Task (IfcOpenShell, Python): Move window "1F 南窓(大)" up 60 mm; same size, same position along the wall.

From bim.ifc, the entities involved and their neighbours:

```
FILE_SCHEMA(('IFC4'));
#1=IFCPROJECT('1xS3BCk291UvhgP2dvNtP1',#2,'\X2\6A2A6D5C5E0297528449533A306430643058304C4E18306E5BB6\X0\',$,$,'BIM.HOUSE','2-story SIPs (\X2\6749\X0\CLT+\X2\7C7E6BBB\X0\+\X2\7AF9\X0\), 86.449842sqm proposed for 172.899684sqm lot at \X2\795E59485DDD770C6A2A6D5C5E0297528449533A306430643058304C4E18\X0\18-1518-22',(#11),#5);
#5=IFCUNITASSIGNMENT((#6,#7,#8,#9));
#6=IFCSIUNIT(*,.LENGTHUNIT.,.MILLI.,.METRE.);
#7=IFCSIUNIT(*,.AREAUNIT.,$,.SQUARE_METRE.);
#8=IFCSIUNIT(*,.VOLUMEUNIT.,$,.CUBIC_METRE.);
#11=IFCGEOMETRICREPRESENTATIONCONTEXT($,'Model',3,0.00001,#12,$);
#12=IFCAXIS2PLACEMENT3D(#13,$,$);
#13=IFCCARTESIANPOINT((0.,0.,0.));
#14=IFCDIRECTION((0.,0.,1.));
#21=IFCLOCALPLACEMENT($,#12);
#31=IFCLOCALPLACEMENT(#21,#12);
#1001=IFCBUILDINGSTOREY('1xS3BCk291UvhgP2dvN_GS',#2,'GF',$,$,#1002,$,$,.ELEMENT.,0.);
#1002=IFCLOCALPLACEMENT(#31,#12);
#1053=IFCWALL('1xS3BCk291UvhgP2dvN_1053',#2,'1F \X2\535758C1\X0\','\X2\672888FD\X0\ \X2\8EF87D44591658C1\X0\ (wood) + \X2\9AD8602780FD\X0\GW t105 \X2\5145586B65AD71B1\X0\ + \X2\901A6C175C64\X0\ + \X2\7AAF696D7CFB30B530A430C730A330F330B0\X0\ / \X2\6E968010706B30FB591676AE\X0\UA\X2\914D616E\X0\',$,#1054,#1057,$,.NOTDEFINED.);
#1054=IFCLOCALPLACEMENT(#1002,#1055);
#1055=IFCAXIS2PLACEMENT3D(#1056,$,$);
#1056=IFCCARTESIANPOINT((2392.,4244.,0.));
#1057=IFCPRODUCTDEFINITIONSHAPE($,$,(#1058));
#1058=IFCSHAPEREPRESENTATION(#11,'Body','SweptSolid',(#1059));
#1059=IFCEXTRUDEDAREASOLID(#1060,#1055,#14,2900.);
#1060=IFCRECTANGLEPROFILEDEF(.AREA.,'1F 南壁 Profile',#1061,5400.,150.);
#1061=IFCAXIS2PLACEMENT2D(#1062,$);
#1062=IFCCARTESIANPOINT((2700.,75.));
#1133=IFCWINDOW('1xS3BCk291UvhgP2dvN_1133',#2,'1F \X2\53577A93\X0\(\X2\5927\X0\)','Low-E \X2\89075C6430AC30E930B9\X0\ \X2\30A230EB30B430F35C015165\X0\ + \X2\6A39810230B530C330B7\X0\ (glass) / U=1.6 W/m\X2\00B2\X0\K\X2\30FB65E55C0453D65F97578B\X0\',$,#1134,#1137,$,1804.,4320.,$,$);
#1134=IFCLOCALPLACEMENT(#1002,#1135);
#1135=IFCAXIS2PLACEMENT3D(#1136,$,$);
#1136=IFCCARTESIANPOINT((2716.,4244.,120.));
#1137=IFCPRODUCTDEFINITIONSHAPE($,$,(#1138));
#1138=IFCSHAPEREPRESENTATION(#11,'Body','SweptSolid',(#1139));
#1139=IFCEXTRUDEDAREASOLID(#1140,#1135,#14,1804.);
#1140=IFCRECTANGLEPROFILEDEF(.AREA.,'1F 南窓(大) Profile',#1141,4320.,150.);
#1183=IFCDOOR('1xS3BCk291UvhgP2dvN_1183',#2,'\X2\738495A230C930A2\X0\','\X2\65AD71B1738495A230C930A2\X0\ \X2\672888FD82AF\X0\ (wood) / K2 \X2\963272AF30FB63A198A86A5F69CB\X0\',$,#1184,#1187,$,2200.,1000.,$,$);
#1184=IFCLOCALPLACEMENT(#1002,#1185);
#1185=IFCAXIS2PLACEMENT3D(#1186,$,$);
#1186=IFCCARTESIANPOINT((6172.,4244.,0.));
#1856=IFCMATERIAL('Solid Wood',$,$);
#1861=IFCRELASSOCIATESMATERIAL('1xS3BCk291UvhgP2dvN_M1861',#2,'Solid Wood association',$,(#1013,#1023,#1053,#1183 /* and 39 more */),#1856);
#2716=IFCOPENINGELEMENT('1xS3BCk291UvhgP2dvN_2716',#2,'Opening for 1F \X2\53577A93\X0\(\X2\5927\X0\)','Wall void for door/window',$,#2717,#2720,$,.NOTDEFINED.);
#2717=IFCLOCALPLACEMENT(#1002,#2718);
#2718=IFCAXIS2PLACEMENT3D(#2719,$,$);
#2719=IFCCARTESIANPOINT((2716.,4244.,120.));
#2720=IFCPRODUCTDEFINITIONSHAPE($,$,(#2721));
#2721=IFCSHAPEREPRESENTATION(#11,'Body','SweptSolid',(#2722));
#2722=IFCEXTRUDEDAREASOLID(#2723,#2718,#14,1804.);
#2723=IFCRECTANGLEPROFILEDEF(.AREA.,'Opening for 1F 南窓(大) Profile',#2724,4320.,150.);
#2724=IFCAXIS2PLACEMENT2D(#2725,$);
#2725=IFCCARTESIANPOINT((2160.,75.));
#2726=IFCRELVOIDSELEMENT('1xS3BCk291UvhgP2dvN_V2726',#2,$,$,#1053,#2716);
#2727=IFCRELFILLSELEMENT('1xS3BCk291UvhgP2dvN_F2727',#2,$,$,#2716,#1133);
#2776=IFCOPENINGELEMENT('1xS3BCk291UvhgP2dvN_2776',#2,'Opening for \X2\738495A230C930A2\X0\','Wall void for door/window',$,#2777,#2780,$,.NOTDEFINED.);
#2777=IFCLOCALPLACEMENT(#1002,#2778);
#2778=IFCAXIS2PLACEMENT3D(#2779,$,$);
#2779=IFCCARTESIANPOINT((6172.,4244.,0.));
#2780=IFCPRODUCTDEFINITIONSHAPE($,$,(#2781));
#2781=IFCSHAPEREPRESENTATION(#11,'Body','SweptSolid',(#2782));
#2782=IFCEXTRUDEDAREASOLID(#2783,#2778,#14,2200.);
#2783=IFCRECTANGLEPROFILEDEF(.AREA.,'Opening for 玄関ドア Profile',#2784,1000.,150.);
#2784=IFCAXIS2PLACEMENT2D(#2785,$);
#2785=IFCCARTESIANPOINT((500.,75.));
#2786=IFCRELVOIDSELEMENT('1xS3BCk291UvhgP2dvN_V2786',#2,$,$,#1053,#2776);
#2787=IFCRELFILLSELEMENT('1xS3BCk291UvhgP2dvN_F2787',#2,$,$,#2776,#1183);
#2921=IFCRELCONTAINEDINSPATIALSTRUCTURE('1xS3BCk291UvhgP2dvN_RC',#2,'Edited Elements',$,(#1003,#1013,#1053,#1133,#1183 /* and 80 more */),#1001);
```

```python
import numpy as np
import ifcopenshell
import ifcopenshell.api.geometry
import ifcopenshell.util.placement
import ifcopenshell.util.unit

model = ifcopenshell.open("bim.ifc")
unit_scale = ifcopenshell.util.unit.calculate_unit_scale(model)

window = model.by_guid("1xS3BCk291UvhgP2dvN_1133")
opening = window.FillsVoids[0].RelatingOpeningElement
dz = 60.0

shift = np.array([0.0, 0.0, dz])
# The window is not placed relative to its opening, so move both.
for product in (opening, window):
    matrix = ifcopenshell.util.placement.get_local_placement(product.ObjectPlacement)
    matrix[:3, 3] += shift
    ifcopenshell.api.geometry.edit_object_placement(model, product=product, matrix=matrix, is_si=False)

print(f"moved by {dz * unit_scale:+.3f} m")

model.write("bim_updated.ifc")
```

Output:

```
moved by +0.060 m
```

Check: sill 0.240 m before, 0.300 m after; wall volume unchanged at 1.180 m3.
